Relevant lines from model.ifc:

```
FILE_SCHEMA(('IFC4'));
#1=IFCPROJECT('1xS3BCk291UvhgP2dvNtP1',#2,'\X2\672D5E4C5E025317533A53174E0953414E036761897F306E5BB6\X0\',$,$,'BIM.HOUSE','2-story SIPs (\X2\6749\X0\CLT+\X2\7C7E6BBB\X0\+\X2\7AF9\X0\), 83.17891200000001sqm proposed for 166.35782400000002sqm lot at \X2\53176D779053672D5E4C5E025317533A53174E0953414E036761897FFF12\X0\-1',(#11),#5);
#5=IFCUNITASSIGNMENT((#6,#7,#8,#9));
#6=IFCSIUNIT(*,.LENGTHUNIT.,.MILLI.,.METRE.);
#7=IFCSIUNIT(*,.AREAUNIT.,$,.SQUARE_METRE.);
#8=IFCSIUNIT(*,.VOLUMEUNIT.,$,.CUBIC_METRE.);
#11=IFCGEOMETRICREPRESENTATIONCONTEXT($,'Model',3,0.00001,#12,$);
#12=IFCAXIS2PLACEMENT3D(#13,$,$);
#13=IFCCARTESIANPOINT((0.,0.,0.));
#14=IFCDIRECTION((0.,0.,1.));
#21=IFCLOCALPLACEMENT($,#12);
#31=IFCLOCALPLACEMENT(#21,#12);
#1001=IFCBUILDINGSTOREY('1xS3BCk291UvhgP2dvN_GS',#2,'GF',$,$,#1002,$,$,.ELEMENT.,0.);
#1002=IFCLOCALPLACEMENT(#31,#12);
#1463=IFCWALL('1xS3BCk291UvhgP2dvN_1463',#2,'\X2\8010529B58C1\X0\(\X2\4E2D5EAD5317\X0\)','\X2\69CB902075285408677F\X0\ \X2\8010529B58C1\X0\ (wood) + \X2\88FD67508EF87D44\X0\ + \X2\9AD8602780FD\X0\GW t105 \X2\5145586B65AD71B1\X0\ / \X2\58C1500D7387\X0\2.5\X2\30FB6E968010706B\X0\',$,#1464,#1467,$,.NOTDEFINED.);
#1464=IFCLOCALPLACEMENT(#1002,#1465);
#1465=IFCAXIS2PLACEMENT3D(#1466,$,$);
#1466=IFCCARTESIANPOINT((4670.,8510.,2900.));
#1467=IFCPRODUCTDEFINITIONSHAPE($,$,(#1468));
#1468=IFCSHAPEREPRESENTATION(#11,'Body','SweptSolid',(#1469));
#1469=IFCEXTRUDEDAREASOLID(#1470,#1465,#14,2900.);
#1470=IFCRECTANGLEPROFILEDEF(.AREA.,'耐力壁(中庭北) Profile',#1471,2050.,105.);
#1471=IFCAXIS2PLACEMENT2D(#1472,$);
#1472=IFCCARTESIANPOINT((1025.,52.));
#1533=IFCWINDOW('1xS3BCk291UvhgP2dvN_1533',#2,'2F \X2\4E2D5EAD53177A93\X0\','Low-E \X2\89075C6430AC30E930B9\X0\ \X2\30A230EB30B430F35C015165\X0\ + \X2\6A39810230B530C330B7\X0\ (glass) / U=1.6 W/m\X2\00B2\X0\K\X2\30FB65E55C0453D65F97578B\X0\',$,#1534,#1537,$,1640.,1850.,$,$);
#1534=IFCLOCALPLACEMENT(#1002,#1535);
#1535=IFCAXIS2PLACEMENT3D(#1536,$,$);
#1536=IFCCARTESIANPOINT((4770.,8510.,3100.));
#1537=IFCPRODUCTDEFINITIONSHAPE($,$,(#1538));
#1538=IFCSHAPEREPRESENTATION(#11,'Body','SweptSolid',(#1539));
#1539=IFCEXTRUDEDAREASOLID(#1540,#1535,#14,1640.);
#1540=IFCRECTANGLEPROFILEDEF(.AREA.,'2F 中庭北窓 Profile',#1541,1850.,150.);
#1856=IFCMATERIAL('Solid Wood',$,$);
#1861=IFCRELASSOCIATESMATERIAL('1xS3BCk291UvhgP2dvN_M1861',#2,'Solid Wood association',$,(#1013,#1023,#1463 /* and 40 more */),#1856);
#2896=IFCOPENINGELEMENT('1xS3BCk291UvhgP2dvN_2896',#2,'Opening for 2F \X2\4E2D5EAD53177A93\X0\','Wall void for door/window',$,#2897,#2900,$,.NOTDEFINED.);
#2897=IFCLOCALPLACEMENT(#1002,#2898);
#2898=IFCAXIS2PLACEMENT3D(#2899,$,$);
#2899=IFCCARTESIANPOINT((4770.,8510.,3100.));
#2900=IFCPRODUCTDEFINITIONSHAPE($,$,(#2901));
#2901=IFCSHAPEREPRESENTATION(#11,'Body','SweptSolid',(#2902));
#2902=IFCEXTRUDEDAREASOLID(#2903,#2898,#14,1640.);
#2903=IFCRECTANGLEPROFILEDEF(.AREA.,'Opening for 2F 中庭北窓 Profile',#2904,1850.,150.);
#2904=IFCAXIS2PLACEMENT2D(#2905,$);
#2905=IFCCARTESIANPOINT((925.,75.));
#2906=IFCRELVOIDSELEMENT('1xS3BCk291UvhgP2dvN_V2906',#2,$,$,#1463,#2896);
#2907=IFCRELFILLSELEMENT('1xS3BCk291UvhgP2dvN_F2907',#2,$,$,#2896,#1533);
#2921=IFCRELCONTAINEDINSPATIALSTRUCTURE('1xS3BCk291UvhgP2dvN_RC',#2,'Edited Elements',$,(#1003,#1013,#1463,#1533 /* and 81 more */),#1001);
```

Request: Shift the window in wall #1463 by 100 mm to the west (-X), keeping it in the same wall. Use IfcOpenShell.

```python
import ifcopenshell
import ifcopenshell.api.geometry
import ifcopenshell.util.placement

model = ifcopenshell.open("model.ifc")

window = model.by_guid("1xS3BCk291UvhgP2dvN_1533")
opening = window.FillsVoids[0].RelatingOpeningElement
wall = opening.VoidsElements[0].RelatingBuildingElement

wall_matrix = ifcopenshell.util.placement.get_local_placement(wall.ObjectPlacement)
shift = wall_matrix[:3, 0] * -100.0
before = ifcopenshell.util.placement.get_local_placement(window.ObjectPlacement)[:3, 3].copy()

# The window is not placed relative to its opening, so move both.
for product in (opening, window):
    matrix = ifcopenshell.util.placement.get_local_placement(product.ObjectPlacement)
    matrix[:3, 3] += shift
    ifcopenshell.api.geometry.edit_object_placement(model, product=product, matrix=matrix, is_si=False)

after = ifcopenshell.util.placement.get_local_placement(window.ObjectPlacement)[:3, 3]
print("window moved by", (after - before).round(3) + 0.0)

model.write("model_edited.ifc")
```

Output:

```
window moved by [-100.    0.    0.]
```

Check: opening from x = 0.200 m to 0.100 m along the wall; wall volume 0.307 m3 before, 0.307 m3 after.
